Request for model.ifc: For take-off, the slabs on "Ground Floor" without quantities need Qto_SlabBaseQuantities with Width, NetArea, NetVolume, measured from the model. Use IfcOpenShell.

First a look at what the model holds.

```python
import ifcopenshell
import ifcopenshell.util.element
import ifcopenshell.util.unit

model = ifcopenshell.open("model.ifc")
print(model.schema)
for unit_type in ("LENGTHUNIT", "AREAUNIT", "VOLUMEUNIT"):
    print(unit_type, ifcopenshell.util.unit.calculate_unit_scale(model, unit_type))
storey = next(s for s in model.by_type("IfcBuildingStorey") if s.Name == "Ground Floor")
slabs = [e for e in ifcopenshell.util.element.get_decomposition(storey) if e.is_a("IfcSlab")]
for e in sorted(slabs, key=lambda e: e.id()):
    print(e.id(), e.is_a(), e.Name, list(ifcopenshell.util.element.get_psets(e, qtos_only=True)), sep=" | ")
```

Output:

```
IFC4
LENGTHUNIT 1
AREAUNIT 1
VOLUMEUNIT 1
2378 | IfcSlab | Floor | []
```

```python
import ifcopenshell
import ifcopenshell.api.pset
import ifcopenshell.geom
import ifcopenshell.util.element
import ifcopenshell.util.shape
import ifcopenshell.util.unit

model = ifcopenshell.open("model.ifc")
unit_scale = ifcopenshell.util.unit.calculate_unit_scale(model)
area_scale = ifcopenshell.util.unit.calculate_unit_scale(model, "AREAUNIT")
volume_scale = ifcopenshell.util.unit.calculate_unit_scale(model, "VOLUMEUNIT")
settings = ifcopenshell.geom.settings()

storey = next(s for s in model.by_type("IfcBuildingStorey") if s.Name == "Ground Floor")
slabs = [e for e in ifcopenshell.util.element.get_decomposition(storey) if e.is_a("IfcSlab")]

for e in sorted(slabs, key=lambda e: e.id()):
    if ifcopenshell.util.element.get_psets(e, qtos_only=True, should_inherit=False):
        continue
    # Geometry comes back in metres, in the element's own axes.
    shape = ifcopenshell.geom.create_shape(settings, e)
    values = {
        "Width": ifcopenshell.util.shape.get_z(shape.geometry) / unit_scale,
        "NetArea": ifcopenshell.util.shape.get_footprint_area(shape.geometry) / area_scale,
        "NetVolume": ifcopenshell.util.shape.get_volume(shape.geometry) / volume_scale,
    }
    qto = ifcopenshell.api.pset.add_qto(model, product=e, name="Qto_SlabBaseQuantities")
    ifcopenshell.api.pset.edit_qto(model, qto=qto, properties=values)
    print(e.id(), {k: round(v, 3) for k, v in values.items()})

model.write("model-out.ifc")
```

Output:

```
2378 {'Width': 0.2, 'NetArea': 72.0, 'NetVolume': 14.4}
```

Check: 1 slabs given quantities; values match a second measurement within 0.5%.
